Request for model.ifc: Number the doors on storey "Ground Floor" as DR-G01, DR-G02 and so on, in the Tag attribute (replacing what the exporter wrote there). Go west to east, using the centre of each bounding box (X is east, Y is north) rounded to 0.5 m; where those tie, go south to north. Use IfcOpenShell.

First a look at what the model holds.

```python
import ifcopenshell
import ifcopenshell.util.element
import ifcopenshell.util.placement

model = ifcopenshell.open("model.ifc")
print(model.schema)
storey = next(s for s in model.by_type("IfcBuildingStorey") if s.Name == "Ground Floor")
doors = [e for e in ifcopenshell.util.element.get_decomposition(storey) if e.is_a("IfcDoor")]
for e in sorted(doors, key=lambda e: e.id()):
    origin = ifcopenshell.util.placement.get_local_placement(e.ObjectPlacement)[:3, 3]
    print(e.id(), e.Tag, e.Name, origin.round(2) + 0.0, sep=" | ")
```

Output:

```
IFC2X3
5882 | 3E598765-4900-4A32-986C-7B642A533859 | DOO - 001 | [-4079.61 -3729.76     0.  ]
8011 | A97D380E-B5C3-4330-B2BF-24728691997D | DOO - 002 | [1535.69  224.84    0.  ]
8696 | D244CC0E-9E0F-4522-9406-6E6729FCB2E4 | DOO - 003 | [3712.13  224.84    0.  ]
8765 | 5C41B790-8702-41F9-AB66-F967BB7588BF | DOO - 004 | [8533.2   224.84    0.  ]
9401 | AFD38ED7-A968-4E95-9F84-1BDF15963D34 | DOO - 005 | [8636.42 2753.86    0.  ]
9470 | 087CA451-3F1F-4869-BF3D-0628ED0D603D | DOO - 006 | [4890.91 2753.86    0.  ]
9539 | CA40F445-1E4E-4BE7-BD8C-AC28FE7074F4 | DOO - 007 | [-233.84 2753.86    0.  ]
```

```python
import ifcopenshell
import ifcopenshell.geom
import ifcopenshell.util.element
import ifcopenshell.util.shape

model = ifcopenshell.open("model.ifc")
settings = ifcopenshell.geom.settings()
settings.set("use-world-coords", True)


def centre(element):
    shape = ifcopenshell.geom.create_shape(settings, element)
    return ifcopenshell.util.shape.get_bbox_centroid(shape.geometry)


storey = next(s for s in model.by_type("IfcBuildingStorey") if s.Name == "Ground Floor")
doors = [e for e in ifcopenshell.util.element.get_decomposition(storey) if e.is_a("IfcDoor")]

# Insertion points can sit at a corner or the storey origin, so sort by the geometry (in metres).
centres = {e: centre(e) for e in doors}
doors.sort(key=lambda e: (round(centres[e][0] / 0.5), centres[e][1]))

for i, e in enumerate(doors, start=1):
    number = f"DR-G{i:02d}"
    e.Tag = number
    print(e.id(), number)

model.write("model_v2.ifc")
```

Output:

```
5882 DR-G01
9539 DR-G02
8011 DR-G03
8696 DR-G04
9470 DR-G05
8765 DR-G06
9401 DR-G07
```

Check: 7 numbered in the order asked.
